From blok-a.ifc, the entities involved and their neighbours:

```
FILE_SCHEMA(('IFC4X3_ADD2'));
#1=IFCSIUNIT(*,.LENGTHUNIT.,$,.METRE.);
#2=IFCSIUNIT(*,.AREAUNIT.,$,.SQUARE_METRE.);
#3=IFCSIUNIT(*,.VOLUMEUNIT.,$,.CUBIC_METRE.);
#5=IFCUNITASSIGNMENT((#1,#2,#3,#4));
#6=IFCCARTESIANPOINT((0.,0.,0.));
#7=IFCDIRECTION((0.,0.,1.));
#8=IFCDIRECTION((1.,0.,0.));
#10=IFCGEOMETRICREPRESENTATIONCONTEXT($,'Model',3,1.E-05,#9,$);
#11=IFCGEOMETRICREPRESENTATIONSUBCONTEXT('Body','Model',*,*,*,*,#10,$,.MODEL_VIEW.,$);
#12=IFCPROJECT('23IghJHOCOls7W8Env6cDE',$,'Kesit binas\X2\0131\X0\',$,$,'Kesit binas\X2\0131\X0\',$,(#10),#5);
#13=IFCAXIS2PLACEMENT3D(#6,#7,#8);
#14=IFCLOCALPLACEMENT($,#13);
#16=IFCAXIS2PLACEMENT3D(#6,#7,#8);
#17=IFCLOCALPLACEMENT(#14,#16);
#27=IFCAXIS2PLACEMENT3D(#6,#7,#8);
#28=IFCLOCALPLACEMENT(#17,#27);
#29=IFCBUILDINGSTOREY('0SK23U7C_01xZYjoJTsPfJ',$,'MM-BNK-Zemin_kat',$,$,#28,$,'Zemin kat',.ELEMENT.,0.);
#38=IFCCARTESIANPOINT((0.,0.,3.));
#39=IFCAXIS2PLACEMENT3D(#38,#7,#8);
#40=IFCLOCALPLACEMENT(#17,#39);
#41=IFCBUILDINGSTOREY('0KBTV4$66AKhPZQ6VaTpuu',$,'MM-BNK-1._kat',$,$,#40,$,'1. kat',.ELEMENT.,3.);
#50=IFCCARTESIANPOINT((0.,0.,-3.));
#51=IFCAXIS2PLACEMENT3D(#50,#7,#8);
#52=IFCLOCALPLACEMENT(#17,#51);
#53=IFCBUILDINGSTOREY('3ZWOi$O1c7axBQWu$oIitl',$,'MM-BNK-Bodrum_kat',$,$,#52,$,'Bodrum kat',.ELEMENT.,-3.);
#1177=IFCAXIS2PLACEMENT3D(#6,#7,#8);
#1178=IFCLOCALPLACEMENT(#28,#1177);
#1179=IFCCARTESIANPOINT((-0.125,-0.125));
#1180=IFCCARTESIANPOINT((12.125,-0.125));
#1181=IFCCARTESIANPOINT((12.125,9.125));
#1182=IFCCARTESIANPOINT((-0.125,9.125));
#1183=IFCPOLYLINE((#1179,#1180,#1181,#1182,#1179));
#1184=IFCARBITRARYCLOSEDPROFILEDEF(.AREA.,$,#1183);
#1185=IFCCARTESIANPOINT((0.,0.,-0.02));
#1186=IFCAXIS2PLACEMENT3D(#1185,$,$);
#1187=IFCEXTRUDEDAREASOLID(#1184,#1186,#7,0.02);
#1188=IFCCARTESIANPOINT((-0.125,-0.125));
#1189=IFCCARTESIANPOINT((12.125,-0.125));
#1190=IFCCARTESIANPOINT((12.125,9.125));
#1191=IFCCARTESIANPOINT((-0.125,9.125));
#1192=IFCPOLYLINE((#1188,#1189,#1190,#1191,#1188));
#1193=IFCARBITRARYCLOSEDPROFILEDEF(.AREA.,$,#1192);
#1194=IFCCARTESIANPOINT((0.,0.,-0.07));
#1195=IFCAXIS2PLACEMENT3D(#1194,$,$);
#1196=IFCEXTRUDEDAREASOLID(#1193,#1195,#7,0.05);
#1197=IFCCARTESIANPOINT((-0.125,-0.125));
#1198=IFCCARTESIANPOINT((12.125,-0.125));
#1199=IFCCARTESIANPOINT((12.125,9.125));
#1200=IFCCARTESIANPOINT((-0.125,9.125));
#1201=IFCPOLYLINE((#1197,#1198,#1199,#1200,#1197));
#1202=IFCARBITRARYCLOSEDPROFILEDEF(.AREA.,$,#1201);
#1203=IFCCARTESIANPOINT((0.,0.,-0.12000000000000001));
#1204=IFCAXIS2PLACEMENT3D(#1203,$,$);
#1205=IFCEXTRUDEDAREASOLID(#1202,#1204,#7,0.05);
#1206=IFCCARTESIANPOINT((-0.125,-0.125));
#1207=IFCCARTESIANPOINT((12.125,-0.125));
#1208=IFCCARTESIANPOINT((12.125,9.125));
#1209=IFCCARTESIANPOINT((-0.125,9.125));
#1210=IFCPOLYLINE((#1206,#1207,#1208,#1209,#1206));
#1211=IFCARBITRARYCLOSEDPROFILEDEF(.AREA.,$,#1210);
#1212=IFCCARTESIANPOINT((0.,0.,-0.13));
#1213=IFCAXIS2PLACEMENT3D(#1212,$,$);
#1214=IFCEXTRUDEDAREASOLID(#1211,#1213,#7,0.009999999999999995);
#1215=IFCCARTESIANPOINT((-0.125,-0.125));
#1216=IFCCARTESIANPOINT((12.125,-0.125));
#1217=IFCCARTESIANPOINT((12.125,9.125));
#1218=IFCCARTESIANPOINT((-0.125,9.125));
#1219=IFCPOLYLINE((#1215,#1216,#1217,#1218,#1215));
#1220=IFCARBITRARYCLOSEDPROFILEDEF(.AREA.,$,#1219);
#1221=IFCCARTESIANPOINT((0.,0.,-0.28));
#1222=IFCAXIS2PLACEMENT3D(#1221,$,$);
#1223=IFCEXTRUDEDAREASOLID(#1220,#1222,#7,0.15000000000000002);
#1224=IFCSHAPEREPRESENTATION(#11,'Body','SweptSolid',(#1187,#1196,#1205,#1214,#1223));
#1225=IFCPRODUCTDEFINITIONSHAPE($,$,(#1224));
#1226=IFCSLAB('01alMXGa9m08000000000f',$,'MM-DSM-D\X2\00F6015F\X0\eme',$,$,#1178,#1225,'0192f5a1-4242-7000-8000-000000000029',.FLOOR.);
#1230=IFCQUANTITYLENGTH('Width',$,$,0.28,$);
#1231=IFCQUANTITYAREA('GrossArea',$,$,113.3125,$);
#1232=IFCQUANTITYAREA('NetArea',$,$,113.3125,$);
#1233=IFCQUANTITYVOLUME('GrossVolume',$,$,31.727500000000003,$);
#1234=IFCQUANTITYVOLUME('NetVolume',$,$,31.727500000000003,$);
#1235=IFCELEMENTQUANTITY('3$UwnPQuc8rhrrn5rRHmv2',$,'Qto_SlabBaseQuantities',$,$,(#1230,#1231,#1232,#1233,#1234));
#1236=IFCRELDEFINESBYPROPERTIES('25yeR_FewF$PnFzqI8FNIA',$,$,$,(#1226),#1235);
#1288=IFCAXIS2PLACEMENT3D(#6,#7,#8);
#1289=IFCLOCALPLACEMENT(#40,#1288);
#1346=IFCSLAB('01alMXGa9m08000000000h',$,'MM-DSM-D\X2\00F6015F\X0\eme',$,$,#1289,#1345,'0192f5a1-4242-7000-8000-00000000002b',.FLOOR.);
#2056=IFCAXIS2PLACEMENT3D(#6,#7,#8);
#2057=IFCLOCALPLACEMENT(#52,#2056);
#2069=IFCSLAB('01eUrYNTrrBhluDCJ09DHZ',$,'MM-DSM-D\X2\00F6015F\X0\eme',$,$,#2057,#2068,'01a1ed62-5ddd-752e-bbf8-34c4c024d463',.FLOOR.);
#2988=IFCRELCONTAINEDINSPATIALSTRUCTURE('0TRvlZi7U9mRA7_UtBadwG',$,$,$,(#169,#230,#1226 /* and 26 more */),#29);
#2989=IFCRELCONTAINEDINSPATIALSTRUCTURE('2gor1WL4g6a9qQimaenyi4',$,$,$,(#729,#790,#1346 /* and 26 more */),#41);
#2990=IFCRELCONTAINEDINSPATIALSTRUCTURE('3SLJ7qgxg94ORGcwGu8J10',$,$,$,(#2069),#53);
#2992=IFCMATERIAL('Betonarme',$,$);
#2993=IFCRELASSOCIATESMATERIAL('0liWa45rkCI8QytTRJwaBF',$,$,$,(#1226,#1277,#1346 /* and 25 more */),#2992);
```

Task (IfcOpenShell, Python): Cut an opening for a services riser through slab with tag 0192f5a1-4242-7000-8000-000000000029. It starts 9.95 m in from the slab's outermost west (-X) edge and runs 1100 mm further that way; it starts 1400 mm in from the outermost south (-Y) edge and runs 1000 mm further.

```python
import numpy as np
import ifcopenshell
import ifcopenshell.api.feature
import ifcopenshell.api.geometry
import ifcopenshell.api.pset
import ifcopenshell.api.root
import ifcopenshell.geom
import ifcopenshell.util.element
import ifcopenshell.util.placement
import ifcopenshell.util.representation
import ifcopenshell.util.shape
import ifcopenshell.util.unit

model = ifcopenshell.open("blok-a.ifc")
unit_scale = ifcopenshell.util.unit.calculate_unit_scale(model)
area_scale = ifcopenshell.util.unit.calculate_unit_scale(model, "AREAUNIT")
volume_scale = ifcopenshell.util.unit.calculate_unit_scale(model, "VOLUMEUNIT")
settings = ifcopenshell.geom.settings()


def volume(element):
    """Net volume in cubic metres, openings subtracted."""
    shape = ifcopenshell.geom.create_shape(settings, element)
    return ifcopenshell.util.shape.get_volume(shape.geometry)


slab = model.by_id(1226)
before = volume(slab)

# Extent in the slab's own axes, in metres. The edges named are its -X and -Y sides.
slab_shape = ifcopenshell.geom.create_shape(settings, slab)
vertices = ifcopenshell.util.shape.get_vertices(slab_shape.geometry)
x_min, y_min, bottom = vertices.min(axis=0)
top = vertices[:, 2].max()

opening = ifcopenshell.api.root.create_entity(model, ifc_class="IfcOpeningElement", name="Services riser opening", predefined_type="OPENING")
context = ifcopenshell.util.representation.get_context(model, "Model", "Body", "MODEL_VIEW")
width, depth = 1.1, 1
outline = [(0.0, 0.0), (width, 0.0), (width, depth), (0.0, depth), (0.0, 0.0)]
# Overshoot both faces by 50 mm so the cut is clean.
shape = ifcopenshell.api.geometry.add_slab_representation(
    model, context=context, depth=top - bottom + 0.1, polyline=outline
)
ifcopenshell.api.geometry.assign_representation(model, product=opening, representation=shape)

matrix = ifcopenshell.util.placement.get_local_placement(slab.ObjectPlacement)
matrix[:, 3] = matrix @ np.append(np.array([x_min + 9.95, y_min + 1.4, bottom - 0.05]) / unit_scale, 1.0)
ifcopenshell.api.geometry.edit_object_placement(model, product=opening, matrix=matrix, is_si=False)
ifcopenshell.api.feature.add_feature(model, feature=opening, element=slab)

after = volume(slab)

# Update the slab's stored quantities.
qto = model.by_id(ifcopenshell.util.element.get_pset(slab, "Qto_SlabBaseQuantities", should_inherit=False)["id"])
ifcopenshell.api.pset.edit_qto(model, qto=qto, properties={
    "NetArea": after / (top - bottom) / area_scale,
    "NetVolume": after / volume_scale,
})

print(f"slab volume {before:.3f} -> {after:.3f} m3")

model.write("blok-a_updated.ifc")
```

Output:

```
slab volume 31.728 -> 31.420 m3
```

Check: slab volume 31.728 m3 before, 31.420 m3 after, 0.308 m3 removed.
